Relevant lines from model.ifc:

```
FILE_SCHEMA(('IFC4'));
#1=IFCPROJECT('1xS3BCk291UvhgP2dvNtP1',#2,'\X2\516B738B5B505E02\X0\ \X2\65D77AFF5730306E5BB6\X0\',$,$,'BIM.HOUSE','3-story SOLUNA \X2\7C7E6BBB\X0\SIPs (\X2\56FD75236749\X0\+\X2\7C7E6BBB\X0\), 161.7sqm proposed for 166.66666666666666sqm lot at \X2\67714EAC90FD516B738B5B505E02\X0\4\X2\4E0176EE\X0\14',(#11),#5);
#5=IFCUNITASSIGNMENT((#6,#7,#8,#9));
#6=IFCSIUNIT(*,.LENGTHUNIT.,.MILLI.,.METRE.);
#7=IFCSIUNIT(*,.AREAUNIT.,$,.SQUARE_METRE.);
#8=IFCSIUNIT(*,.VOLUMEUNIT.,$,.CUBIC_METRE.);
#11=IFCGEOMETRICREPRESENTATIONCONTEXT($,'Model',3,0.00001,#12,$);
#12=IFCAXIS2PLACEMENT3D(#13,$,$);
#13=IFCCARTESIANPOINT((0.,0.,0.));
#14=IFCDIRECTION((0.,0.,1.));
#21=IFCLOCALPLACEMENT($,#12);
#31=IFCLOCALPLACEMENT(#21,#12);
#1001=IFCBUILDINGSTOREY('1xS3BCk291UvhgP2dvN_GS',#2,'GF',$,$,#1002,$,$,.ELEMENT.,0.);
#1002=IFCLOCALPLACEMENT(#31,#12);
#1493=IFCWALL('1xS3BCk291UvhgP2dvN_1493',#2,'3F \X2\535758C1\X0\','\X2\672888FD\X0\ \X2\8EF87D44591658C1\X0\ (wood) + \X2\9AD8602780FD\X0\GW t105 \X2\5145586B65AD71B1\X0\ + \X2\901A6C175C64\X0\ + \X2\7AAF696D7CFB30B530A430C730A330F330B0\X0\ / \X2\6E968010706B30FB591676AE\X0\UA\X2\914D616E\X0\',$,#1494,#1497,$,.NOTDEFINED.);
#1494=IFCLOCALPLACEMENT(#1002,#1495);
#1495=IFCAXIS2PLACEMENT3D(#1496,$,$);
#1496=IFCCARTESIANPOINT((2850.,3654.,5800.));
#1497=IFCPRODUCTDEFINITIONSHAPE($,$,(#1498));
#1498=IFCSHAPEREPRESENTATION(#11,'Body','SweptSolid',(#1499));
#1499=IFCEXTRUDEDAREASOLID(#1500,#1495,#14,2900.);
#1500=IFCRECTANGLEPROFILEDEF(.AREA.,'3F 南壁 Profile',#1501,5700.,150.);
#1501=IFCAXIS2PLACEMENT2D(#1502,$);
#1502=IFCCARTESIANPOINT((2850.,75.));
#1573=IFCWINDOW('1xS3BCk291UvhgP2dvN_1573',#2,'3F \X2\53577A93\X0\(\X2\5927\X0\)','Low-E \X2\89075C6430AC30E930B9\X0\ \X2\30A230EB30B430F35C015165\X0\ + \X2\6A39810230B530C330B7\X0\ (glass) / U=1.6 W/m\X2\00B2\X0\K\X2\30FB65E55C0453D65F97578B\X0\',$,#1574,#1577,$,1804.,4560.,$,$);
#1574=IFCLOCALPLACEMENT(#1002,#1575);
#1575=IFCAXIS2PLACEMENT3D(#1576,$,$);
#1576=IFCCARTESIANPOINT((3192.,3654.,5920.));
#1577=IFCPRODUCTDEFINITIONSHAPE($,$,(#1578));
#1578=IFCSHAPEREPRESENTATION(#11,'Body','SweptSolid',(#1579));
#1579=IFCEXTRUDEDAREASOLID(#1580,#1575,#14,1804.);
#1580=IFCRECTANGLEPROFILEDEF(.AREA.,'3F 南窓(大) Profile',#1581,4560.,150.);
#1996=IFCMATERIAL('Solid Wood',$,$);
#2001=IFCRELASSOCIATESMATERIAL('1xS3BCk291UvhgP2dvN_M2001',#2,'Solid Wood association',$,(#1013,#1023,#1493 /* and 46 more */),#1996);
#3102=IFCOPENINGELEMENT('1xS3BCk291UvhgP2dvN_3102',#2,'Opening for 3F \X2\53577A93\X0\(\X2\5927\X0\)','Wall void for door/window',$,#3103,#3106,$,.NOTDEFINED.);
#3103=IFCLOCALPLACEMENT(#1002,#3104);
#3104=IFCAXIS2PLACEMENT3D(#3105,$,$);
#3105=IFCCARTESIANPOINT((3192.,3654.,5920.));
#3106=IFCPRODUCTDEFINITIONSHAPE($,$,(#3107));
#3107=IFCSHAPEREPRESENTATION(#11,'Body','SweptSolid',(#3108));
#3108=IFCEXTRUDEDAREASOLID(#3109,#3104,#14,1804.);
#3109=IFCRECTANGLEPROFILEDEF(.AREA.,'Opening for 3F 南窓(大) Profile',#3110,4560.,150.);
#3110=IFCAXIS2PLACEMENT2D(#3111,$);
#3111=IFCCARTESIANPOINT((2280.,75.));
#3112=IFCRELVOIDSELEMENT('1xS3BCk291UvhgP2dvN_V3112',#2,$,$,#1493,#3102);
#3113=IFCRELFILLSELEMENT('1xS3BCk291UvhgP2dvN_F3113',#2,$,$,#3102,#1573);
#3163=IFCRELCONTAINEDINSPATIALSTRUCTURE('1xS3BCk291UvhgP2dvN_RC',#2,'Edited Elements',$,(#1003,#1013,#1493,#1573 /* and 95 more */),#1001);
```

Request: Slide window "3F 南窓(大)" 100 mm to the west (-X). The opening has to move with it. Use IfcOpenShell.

```python
import ifcopenshell
import ifcopenshell.api.geometry
import ifcopenshell.util.placement
import ifcopenshell.util.unit

model = ifcopenshell.open("model.ifc")
unit_scale = ifcopenshell.util.unit.calculate_unit_scale(model)

window = model.by_id(1573)
opening = window.FillsVoids[0].RelatingOpeningElement
wall = opening.VoidsElements[0].RelatingBuildingElement

wall_matrix = ifcopenshell.util.placement.get_local_placement(wall.ObjectPlacement)
shift = wall_matrix[:3, 0] * -0.1 / unit_scale
before = ifcopenshell.util.placement.get_local_placement(window.ObjectPlacement)[:3, 3].copy()

# The window is not placed relative to its opening, so move both.
for product in (opening, window):
    matrix = ifcopenshell.util.placement.get_local_placement(product.ObjectPlacement)
    matrix[:3, 3] += shift
    ifcopenshell.api.geometry.edit_object_placement(model, product=product, matrix=matrix, is_si=False)

after = ifcopenshell.util.placement.get_local_placement(window.ObjectPlacement)[:3, 3]
print("window moved by", (after - before).round(3) + 0.0)

model.write("model_updated.ifc")
```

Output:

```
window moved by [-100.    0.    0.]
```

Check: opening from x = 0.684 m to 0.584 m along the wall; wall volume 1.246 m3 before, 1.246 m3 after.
